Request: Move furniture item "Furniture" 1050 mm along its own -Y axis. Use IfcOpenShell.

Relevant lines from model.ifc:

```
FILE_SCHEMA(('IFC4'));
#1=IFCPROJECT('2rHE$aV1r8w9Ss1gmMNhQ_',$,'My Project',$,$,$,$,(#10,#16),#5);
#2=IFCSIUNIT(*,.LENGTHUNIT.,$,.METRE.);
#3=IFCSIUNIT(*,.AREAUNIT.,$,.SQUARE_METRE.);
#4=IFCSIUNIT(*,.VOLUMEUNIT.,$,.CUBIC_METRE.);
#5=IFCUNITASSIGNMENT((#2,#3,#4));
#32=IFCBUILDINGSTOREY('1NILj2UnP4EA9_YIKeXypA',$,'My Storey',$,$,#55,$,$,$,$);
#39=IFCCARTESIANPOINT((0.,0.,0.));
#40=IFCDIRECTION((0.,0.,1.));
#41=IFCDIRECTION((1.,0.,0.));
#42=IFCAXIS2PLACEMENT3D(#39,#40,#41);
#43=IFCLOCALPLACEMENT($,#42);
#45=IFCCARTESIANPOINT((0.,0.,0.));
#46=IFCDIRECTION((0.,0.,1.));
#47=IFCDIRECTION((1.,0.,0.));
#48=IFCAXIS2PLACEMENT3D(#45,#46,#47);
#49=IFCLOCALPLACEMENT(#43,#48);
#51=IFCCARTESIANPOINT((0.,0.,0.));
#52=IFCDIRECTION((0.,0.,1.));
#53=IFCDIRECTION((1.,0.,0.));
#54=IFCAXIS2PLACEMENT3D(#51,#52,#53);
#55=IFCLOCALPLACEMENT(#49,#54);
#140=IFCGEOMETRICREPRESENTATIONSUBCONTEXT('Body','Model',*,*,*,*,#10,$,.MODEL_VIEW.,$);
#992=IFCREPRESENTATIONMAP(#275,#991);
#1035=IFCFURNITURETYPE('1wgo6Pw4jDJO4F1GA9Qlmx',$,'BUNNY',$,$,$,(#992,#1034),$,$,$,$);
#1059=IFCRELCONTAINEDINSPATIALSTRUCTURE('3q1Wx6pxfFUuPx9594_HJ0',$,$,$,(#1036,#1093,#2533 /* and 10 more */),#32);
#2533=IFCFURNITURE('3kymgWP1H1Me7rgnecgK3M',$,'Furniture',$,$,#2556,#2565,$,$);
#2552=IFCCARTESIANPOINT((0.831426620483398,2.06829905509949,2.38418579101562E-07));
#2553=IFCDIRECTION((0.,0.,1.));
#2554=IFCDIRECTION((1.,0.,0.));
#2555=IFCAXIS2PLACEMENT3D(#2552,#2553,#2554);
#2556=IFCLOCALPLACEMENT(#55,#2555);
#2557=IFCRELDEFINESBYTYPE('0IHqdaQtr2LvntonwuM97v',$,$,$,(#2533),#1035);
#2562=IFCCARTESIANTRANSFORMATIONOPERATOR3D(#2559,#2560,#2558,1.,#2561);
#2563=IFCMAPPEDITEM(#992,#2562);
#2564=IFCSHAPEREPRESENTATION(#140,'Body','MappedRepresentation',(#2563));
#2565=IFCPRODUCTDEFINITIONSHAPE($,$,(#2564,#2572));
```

```python
import ifcopenshell
import ifcopenshell.api.geometry
import ifcopenshell.util.placement

model = ifcopenshell.open("model.ifc")

item = model.by_guid("3kymgWP1H1Me7rgnecgK3M")
matrix = ifcopenshell.util.placement.get_local_placement(item.ObjectPlacement)
matrix[:3, 3] -= matrix[:3, 1] * 1.05
ifcopenshell.api.geometry.edit_object_placement(model, product=item, matrix=matrix, is_si=False)

print(ifcopenshell.util.placement.get_local_placement(item.ObjectPlacement).round(3) + 0.0)

model.write("model_updated.ifc")
```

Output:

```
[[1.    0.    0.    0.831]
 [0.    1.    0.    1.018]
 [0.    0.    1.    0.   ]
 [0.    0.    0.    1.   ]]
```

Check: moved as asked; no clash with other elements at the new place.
